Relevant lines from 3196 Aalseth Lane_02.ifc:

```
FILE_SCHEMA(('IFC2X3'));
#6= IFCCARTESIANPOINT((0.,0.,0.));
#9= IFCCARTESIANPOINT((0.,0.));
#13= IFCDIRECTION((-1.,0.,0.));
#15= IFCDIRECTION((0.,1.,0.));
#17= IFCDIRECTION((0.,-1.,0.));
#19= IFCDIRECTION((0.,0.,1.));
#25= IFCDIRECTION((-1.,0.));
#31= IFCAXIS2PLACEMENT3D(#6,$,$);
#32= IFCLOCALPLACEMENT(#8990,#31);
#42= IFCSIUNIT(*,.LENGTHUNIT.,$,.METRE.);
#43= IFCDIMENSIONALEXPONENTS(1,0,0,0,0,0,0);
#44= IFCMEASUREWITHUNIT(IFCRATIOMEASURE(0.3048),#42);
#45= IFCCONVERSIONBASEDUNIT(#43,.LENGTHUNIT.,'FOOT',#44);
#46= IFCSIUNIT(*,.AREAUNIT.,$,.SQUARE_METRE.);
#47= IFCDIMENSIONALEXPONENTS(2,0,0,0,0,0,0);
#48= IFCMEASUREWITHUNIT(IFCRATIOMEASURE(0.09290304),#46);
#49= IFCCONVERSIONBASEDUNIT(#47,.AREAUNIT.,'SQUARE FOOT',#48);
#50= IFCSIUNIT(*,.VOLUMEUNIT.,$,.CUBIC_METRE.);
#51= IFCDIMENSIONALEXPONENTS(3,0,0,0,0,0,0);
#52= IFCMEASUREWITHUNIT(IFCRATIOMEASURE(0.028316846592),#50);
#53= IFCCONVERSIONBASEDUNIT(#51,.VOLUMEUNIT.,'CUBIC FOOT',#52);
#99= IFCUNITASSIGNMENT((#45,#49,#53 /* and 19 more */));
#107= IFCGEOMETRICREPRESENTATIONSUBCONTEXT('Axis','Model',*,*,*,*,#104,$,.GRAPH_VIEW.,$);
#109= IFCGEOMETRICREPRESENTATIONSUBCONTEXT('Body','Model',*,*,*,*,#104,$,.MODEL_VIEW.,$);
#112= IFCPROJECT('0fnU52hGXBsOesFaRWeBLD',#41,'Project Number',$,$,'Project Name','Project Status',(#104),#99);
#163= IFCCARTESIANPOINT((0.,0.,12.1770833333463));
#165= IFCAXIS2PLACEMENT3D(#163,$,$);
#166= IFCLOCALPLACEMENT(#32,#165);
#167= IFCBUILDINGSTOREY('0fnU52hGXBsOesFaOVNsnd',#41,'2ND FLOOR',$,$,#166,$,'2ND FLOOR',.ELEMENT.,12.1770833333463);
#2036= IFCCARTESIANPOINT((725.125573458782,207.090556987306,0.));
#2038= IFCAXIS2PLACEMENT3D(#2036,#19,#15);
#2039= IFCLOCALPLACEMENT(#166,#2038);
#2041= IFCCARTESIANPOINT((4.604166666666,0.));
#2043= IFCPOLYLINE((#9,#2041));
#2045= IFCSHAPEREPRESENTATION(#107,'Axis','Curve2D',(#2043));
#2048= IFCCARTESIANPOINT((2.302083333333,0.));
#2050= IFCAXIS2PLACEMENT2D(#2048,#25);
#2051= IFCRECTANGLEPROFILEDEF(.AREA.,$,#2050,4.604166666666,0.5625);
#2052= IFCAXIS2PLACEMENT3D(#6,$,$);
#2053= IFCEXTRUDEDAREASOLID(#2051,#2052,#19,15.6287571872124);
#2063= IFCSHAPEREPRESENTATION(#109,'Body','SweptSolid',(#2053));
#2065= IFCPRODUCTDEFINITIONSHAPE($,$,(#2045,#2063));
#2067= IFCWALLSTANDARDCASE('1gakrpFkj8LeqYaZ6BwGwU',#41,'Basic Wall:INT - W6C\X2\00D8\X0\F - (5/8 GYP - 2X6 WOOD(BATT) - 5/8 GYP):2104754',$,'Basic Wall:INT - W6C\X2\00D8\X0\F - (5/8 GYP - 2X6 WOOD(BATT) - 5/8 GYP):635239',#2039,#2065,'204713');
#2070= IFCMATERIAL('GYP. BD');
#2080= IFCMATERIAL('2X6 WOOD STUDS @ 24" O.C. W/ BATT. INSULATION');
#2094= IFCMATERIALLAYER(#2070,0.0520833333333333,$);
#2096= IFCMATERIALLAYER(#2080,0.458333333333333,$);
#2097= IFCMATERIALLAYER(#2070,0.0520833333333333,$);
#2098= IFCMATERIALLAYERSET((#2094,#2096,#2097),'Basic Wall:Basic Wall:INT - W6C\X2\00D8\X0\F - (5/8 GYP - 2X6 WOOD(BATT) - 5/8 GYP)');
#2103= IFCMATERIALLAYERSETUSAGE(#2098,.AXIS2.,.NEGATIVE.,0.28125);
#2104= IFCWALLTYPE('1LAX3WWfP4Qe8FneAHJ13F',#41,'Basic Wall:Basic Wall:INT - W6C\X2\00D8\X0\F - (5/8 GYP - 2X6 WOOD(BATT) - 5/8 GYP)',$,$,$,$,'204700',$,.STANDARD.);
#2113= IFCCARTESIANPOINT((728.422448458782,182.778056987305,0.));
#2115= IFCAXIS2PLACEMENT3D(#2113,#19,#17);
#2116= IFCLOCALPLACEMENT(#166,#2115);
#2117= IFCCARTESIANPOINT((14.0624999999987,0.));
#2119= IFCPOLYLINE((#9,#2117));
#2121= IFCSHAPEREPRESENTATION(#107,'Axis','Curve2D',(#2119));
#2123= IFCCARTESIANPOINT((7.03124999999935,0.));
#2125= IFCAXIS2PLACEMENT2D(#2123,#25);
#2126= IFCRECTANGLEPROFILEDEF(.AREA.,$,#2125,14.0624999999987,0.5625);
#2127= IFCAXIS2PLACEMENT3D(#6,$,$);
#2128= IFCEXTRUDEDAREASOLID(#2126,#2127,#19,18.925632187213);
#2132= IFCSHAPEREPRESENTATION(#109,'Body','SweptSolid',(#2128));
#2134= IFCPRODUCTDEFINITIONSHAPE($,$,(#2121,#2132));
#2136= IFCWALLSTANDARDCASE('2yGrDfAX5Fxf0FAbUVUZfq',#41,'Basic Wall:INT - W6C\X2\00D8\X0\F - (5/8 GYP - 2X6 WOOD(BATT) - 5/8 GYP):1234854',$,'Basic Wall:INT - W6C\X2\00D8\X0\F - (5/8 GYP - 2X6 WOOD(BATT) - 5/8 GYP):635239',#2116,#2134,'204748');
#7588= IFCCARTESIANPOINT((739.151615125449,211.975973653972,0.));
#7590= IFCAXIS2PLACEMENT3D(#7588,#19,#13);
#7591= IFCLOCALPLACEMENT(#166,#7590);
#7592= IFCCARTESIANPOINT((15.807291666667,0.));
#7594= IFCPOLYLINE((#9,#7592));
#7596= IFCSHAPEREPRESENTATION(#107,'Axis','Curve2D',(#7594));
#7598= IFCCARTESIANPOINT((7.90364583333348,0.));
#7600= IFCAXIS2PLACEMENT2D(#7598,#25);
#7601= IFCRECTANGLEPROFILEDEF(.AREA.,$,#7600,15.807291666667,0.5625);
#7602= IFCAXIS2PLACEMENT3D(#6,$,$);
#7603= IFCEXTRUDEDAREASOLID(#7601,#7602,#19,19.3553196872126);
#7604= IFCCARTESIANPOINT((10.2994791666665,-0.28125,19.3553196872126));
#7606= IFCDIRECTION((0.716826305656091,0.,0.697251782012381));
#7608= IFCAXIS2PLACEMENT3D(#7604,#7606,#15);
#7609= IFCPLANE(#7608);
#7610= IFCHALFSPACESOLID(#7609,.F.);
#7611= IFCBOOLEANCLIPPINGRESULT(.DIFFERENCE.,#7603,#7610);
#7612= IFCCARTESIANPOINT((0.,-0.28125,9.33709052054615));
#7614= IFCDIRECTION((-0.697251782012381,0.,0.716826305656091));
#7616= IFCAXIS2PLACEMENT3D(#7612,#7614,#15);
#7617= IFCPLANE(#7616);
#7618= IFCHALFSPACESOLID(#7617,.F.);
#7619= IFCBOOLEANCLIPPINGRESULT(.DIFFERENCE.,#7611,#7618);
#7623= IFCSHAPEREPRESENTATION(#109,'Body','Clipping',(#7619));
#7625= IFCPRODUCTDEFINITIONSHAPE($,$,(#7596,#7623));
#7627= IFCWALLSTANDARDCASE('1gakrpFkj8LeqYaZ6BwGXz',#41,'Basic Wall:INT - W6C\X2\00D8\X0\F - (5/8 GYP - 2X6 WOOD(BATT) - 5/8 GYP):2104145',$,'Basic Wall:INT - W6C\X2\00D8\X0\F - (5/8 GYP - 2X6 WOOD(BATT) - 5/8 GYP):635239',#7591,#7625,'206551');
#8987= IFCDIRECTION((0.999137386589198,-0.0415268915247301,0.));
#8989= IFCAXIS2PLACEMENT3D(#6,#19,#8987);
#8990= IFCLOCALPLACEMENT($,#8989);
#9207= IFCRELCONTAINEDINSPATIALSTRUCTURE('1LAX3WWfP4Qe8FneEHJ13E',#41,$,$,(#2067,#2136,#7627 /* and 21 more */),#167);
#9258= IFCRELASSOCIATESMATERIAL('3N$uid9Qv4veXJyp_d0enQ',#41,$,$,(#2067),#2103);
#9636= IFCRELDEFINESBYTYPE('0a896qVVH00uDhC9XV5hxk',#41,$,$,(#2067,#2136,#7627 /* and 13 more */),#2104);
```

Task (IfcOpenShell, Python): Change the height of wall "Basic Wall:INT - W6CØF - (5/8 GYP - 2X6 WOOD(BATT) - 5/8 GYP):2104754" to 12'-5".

```python
import ifcopenshell
import ifcopenshell.geom
import ifcopenshell.util.representation
import ifcopenshell.util.shape
import ifcopenshell.util.unit

model = ifcopenshell.open("3196 Aalseth Lane_02.ifc")
unit_scale = ifcopenshell.util.unit.calculate_unit_scale(model)
settings = ifcopenshell.geom.settings()


def volume(element):
    """Net volume in cubic metres, openings subtracted."""
    shape = ifcopenshell.geom.create_shape(settings, element)
    return ifcopenshell.util.shape.get_volume(shape.geometry)


wall = model.by_id(2067)
before = volume(wall)

body = ifcopenshell.util.representation.get_representation(wall, "Model", "Body")
solid = body.Items[0]
old_height = solid.Depth
solid.Depth = 149 * 0.0254 / unit_scale
after = volume(wall)

print(f"height {old_height:g} -> {solid.Depth:g}, volume {before:.3f} -> {after:.3f} m3")

model.write("3196 Aalseth Lane_02-out.ifc")
```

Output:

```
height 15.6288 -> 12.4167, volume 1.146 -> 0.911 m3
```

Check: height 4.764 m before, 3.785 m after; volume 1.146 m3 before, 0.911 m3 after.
